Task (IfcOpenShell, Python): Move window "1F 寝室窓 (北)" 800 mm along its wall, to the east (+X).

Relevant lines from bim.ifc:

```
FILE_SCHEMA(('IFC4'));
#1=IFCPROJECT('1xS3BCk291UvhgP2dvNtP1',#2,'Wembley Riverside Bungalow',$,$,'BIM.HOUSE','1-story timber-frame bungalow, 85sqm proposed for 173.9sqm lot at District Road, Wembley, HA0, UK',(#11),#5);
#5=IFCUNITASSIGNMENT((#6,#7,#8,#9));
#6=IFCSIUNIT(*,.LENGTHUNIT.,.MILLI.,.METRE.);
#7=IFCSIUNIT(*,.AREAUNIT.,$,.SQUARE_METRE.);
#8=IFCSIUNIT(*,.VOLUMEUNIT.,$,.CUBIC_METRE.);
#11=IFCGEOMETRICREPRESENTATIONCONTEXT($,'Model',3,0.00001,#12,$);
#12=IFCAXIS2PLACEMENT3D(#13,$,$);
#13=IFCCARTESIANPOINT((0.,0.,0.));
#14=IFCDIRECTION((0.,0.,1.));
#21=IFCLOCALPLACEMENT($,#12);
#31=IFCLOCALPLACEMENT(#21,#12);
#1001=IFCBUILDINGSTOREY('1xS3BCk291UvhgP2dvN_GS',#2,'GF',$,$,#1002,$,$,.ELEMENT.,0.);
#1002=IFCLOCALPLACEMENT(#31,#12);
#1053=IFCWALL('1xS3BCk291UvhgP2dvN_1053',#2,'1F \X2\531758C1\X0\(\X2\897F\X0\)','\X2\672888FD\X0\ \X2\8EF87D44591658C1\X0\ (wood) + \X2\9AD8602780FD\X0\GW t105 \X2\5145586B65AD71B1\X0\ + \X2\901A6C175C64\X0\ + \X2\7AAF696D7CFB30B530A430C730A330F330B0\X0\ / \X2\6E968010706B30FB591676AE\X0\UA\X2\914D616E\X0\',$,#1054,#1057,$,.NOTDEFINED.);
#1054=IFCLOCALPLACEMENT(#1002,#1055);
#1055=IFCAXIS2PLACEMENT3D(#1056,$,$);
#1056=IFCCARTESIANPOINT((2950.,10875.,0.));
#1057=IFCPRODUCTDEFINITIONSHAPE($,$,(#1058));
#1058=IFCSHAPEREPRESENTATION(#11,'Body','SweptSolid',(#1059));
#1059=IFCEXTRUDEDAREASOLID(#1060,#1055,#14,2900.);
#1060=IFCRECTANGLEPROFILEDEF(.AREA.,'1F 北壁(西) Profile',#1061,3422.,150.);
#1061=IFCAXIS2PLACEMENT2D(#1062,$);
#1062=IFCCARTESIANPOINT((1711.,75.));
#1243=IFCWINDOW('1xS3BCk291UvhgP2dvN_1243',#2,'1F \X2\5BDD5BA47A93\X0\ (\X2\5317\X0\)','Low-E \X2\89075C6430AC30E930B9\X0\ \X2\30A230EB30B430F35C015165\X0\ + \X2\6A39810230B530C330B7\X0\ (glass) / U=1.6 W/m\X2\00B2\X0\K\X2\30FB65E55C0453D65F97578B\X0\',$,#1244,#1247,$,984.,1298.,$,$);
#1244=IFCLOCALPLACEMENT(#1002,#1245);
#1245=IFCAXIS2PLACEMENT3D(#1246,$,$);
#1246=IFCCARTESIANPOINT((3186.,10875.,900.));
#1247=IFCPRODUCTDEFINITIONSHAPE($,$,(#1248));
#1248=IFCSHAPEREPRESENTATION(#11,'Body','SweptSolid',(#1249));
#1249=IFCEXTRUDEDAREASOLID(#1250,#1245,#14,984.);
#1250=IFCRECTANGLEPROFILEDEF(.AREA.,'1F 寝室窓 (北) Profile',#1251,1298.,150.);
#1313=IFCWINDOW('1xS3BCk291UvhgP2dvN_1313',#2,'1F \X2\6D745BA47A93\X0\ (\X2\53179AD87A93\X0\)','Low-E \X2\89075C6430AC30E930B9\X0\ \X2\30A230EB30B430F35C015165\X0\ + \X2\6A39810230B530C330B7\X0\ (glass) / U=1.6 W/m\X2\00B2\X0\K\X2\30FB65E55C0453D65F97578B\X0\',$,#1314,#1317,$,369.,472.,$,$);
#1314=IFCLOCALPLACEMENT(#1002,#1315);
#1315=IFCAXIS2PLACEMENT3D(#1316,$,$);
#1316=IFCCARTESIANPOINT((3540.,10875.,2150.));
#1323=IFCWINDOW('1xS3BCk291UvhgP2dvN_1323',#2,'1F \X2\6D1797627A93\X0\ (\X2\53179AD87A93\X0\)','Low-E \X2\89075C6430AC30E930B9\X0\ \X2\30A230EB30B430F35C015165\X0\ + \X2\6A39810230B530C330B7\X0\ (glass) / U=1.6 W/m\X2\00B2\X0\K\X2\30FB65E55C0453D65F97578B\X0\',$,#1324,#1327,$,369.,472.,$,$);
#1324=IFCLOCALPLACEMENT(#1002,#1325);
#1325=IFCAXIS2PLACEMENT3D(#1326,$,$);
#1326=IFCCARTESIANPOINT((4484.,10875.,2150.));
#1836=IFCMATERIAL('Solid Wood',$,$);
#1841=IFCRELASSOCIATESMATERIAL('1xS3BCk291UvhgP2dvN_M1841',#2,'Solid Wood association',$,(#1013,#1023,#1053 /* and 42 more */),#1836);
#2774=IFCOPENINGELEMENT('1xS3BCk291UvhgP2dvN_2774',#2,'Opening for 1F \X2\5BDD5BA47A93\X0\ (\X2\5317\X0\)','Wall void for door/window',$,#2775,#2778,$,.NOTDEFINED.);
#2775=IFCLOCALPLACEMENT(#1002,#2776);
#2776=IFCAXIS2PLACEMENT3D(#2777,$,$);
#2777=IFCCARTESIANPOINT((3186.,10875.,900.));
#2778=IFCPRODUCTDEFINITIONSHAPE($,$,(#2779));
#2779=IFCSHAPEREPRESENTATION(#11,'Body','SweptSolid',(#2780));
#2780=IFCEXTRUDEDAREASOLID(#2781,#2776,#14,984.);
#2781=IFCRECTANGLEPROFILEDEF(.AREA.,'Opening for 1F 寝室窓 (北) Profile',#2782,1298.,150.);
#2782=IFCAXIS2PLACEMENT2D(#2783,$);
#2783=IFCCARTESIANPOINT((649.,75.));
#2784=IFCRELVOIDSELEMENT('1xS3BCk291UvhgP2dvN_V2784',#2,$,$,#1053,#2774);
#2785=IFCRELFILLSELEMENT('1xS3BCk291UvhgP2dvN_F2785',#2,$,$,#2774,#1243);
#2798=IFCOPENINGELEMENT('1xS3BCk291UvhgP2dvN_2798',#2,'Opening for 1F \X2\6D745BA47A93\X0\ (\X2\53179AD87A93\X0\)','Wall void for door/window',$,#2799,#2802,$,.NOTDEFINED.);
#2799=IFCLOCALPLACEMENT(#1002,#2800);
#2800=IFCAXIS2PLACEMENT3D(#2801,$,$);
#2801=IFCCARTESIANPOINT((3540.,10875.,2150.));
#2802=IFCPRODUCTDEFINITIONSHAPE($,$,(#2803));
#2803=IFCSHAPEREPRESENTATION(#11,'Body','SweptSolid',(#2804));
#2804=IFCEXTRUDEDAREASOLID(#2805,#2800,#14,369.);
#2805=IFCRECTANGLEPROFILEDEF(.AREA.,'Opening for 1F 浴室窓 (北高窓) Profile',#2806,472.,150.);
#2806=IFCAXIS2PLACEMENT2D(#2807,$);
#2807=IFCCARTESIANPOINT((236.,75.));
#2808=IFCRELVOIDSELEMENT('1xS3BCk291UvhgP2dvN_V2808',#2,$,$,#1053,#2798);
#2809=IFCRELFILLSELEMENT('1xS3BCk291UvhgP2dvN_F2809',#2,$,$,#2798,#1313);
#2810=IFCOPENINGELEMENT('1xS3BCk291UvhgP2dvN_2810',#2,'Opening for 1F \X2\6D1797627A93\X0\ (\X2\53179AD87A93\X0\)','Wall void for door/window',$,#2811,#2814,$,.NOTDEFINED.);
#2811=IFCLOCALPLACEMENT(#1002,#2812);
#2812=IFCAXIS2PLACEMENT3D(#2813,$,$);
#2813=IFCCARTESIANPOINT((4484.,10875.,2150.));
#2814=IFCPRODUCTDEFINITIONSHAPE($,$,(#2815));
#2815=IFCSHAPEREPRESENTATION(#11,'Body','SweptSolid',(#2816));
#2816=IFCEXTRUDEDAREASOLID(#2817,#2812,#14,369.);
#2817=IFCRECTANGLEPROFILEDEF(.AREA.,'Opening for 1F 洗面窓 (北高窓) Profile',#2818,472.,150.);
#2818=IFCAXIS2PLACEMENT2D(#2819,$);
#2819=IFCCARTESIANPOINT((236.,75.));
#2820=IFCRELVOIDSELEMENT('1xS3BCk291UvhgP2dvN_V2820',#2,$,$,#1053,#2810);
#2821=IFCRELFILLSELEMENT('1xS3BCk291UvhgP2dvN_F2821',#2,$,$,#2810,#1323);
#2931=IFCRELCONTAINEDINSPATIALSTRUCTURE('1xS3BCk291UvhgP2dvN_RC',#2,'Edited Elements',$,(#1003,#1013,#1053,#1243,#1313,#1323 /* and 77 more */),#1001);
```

```python
import ifcopenshell
import ifcopenshell.api.geometry
import ifcopenshell.util.placement
import ifcopenshell.util.unit

model = ifcopenshell.open("bim.ifc")
unit_scale = ifcopenshell.util.unit.calculate_unit_scale(model)

window = model.by_id(1243)
opening = window.FillsVoids[0].RelatingOpeningElement
wall = opening.VoidsElements[0].RelatingBuildingElement

wall_matrix = ifcopenshell.util.placement.get_local_placement(wall.ObjectPlacement)
shift = wall_matrix[:3, 0] * 0.8 / unit_scale
before = ifcopenshell.util.placement.get_local_placement(window.ObjectPlacement)[:3, 3].copy()

# The window is not placed relative to its opening, so move both.
for product in (opening, window):
    matrix = ifcopenshell.util.placement.get_local_placement(product.ObjectPlacement)
    matrix[:3, 3] += shift
    ifcopenshell.api.geometry.edit_object_placement(model, product=product, matrix=matrix, is_si=False)

after = ifcopenshell.util.placement.get_local_placement(window.ObjectPlacement)[:3, 3]
print("window moved by", (after - before).round(3) + 0.0)

model.write("bim_v2.ifc")
```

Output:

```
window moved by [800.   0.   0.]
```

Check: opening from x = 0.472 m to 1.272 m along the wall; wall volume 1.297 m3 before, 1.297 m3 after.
